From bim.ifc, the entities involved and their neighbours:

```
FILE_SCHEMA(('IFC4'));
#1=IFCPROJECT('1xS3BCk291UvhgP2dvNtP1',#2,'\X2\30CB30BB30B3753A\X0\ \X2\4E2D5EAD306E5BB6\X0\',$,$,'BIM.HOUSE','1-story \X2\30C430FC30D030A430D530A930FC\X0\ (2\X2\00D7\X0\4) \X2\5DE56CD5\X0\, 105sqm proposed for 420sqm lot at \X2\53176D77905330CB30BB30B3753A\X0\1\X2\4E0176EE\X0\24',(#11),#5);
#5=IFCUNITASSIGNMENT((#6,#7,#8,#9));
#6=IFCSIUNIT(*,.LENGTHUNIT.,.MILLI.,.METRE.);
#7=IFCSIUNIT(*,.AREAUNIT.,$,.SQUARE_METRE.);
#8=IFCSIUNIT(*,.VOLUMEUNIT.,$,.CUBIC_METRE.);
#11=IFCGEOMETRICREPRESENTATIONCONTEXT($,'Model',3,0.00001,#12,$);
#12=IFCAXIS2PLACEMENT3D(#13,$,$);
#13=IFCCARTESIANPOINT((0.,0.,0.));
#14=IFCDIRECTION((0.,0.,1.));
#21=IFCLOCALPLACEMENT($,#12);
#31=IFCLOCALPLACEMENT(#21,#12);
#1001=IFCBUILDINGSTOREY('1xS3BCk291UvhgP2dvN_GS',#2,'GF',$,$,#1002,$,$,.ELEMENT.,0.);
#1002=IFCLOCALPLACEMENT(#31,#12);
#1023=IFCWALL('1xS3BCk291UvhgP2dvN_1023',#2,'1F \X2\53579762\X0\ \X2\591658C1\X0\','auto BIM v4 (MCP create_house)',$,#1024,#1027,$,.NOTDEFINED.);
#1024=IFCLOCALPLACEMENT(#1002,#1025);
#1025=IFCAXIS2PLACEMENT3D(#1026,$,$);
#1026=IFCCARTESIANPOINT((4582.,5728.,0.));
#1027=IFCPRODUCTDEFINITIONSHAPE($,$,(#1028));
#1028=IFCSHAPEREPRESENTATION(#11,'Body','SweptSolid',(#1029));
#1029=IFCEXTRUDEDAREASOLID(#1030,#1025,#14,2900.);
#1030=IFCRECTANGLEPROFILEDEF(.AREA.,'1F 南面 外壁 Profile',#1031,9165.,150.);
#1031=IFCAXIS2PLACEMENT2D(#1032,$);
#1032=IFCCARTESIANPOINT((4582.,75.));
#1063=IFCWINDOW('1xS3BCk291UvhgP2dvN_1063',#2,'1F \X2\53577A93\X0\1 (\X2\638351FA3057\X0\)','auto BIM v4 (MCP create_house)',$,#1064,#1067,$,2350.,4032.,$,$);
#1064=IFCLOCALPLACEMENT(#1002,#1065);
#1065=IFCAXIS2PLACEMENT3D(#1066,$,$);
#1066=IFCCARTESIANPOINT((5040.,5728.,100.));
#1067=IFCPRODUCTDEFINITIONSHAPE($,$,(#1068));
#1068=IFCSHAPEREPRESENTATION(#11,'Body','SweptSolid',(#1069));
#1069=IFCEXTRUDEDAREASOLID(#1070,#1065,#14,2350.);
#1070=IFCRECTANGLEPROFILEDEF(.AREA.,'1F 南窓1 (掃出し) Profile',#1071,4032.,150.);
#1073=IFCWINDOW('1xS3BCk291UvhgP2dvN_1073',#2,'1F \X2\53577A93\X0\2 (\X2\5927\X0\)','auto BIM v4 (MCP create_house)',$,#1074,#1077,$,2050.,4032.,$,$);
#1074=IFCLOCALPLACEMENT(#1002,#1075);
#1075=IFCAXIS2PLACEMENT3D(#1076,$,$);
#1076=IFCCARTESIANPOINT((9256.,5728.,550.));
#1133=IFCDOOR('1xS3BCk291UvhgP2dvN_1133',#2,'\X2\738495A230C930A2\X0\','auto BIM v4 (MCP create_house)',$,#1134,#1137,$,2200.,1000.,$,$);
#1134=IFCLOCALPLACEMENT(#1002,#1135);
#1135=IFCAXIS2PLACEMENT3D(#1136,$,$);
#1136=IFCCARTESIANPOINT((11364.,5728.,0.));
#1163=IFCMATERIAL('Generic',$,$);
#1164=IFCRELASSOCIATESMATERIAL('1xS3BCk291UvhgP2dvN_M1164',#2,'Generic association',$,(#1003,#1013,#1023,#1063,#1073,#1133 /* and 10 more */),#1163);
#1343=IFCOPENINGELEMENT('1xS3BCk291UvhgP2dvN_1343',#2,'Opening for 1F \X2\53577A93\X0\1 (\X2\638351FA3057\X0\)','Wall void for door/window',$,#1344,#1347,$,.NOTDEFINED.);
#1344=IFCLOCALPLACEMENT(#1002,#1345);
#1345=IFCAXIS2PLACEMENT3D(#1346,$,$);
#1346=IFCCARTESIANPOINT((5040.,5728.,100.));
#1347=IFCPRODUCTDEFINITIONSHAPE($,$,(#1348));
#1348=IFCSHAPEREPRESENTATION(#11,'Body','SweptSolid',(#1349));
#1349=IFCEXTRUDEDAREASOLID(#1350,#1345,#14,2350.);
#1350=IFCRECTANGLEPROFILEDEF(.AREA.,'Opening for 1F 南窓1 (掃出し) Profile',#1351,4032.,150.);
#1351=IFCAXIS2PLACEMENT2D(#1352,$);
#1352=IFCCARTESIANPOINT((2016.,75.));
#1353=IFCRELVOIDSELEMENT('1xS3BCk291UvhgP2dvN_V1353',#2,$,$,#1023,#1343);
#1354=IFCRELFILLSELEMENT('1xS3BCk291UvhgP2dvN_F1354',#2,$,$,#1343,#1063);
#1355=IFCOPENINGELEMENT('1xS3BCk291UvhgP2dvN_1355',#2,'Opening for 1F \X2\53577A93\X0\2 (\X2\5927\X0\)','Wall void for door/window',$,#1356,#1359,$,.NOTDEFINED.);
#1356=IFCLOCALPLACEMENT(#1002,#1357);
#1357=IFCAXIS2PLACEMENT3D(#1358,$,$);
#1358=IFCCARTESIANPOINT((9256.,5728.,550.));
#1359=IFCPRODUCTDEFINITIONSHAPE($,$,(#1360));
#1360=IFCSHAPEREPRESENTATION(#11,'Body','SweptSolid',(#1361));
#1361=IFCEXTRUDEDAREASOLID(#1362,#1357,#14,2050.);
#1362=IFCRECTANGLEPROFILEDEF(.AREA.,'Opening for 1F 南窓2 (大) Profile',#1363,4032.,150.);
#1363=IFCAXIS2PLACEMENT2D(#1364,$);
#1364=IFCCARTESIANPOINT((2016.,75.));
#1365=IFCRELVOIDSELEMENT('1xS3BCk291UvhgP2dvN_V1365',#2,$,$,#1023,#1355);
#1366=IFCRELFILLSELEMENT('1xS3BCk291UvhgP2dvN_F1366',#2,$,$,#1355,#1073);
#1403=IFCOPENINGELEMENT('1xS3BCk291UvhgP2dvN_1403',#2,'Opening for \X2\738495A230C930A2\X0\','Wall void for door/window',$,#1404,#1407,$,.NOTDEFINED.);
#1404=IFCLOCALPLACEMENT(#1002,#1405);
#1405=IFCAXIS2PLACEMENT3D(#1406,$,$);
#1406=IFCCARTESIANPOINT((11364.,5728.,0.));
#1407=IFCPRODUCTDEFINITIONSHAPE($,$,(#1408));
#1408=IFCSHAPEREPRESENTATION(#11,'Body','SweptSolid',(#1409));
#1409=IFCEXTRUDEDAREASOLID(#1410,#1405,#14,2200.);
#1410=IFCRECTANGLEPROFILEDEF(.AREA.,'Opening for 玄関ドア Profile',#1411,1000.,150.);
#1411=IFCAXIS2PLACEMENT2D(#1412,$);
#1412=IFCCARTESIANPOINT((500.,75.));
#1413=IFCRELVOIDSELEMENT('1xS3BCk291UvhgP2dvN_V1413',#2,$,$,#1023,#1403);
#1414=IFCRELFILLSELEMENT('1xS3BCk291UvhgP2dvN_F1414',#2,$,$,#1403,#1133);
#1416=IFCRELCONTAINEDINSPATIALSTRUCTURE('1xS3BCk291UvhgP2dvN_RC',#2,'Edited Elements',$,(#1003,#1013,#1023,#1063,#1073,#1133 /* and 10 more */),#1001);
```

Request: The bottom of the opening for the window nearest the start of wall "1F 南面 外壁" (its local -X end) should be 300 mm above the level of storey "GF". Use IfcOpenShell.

```python
import numpy as np
import ifcopenshell
import ifcopenshell.api.geometry
import ifcopenshell.geom
import ifcopenshell.util.element
import ifcopenshell.util.placement
import ifcopenshell.util.shape
import ifcopenshell.util.unit

model = ifcopenshell.open("bim.ifc")
unit_scale = ifcopenshell.util.unit.calculate_unit_scale(model)

window = model.by_id(1063)
opening = window.FillsVoids[0].RelatingOpeningElement
storey = ifcopenshell.util.element.get_container(window, ifc_class="IfcBuildingStorey")
level = ifcopenshell.util.placement.get_local_placement(storey.ObjectPlacement)[2, 3]

# The opening's origin need not be at the sill, so measure its lowest point.
shape = ifcopenshell.geom.create_shape(ifcopenshell.geom.settings(), opening)
bottom = ifcopenshell.util.shape.get_shape_bottom_elevation(shape, shape.geometry) / unit_scale
dz = level + 300.0 - bottom

shift = np.array([0.0, 0.0, dz])
# The window is not placed relative to its opening, so move both.
for product in (opening, window):
    matrix = ifcopenshell.util.placement.get_local_placement(product.ObjectPlacement)
    matrix[:3, 3] += shift
    ifcopenshell.api.geometry.edit_object_placement(model, product=product, matrix=matrix, is_si=False)

print(f"moved by {dz * unit_scale:+.3f} m")

model.write("bim_updated.ifc")
```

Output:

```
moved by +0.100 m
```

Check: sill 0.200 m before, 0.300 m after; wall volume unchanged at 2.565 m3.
